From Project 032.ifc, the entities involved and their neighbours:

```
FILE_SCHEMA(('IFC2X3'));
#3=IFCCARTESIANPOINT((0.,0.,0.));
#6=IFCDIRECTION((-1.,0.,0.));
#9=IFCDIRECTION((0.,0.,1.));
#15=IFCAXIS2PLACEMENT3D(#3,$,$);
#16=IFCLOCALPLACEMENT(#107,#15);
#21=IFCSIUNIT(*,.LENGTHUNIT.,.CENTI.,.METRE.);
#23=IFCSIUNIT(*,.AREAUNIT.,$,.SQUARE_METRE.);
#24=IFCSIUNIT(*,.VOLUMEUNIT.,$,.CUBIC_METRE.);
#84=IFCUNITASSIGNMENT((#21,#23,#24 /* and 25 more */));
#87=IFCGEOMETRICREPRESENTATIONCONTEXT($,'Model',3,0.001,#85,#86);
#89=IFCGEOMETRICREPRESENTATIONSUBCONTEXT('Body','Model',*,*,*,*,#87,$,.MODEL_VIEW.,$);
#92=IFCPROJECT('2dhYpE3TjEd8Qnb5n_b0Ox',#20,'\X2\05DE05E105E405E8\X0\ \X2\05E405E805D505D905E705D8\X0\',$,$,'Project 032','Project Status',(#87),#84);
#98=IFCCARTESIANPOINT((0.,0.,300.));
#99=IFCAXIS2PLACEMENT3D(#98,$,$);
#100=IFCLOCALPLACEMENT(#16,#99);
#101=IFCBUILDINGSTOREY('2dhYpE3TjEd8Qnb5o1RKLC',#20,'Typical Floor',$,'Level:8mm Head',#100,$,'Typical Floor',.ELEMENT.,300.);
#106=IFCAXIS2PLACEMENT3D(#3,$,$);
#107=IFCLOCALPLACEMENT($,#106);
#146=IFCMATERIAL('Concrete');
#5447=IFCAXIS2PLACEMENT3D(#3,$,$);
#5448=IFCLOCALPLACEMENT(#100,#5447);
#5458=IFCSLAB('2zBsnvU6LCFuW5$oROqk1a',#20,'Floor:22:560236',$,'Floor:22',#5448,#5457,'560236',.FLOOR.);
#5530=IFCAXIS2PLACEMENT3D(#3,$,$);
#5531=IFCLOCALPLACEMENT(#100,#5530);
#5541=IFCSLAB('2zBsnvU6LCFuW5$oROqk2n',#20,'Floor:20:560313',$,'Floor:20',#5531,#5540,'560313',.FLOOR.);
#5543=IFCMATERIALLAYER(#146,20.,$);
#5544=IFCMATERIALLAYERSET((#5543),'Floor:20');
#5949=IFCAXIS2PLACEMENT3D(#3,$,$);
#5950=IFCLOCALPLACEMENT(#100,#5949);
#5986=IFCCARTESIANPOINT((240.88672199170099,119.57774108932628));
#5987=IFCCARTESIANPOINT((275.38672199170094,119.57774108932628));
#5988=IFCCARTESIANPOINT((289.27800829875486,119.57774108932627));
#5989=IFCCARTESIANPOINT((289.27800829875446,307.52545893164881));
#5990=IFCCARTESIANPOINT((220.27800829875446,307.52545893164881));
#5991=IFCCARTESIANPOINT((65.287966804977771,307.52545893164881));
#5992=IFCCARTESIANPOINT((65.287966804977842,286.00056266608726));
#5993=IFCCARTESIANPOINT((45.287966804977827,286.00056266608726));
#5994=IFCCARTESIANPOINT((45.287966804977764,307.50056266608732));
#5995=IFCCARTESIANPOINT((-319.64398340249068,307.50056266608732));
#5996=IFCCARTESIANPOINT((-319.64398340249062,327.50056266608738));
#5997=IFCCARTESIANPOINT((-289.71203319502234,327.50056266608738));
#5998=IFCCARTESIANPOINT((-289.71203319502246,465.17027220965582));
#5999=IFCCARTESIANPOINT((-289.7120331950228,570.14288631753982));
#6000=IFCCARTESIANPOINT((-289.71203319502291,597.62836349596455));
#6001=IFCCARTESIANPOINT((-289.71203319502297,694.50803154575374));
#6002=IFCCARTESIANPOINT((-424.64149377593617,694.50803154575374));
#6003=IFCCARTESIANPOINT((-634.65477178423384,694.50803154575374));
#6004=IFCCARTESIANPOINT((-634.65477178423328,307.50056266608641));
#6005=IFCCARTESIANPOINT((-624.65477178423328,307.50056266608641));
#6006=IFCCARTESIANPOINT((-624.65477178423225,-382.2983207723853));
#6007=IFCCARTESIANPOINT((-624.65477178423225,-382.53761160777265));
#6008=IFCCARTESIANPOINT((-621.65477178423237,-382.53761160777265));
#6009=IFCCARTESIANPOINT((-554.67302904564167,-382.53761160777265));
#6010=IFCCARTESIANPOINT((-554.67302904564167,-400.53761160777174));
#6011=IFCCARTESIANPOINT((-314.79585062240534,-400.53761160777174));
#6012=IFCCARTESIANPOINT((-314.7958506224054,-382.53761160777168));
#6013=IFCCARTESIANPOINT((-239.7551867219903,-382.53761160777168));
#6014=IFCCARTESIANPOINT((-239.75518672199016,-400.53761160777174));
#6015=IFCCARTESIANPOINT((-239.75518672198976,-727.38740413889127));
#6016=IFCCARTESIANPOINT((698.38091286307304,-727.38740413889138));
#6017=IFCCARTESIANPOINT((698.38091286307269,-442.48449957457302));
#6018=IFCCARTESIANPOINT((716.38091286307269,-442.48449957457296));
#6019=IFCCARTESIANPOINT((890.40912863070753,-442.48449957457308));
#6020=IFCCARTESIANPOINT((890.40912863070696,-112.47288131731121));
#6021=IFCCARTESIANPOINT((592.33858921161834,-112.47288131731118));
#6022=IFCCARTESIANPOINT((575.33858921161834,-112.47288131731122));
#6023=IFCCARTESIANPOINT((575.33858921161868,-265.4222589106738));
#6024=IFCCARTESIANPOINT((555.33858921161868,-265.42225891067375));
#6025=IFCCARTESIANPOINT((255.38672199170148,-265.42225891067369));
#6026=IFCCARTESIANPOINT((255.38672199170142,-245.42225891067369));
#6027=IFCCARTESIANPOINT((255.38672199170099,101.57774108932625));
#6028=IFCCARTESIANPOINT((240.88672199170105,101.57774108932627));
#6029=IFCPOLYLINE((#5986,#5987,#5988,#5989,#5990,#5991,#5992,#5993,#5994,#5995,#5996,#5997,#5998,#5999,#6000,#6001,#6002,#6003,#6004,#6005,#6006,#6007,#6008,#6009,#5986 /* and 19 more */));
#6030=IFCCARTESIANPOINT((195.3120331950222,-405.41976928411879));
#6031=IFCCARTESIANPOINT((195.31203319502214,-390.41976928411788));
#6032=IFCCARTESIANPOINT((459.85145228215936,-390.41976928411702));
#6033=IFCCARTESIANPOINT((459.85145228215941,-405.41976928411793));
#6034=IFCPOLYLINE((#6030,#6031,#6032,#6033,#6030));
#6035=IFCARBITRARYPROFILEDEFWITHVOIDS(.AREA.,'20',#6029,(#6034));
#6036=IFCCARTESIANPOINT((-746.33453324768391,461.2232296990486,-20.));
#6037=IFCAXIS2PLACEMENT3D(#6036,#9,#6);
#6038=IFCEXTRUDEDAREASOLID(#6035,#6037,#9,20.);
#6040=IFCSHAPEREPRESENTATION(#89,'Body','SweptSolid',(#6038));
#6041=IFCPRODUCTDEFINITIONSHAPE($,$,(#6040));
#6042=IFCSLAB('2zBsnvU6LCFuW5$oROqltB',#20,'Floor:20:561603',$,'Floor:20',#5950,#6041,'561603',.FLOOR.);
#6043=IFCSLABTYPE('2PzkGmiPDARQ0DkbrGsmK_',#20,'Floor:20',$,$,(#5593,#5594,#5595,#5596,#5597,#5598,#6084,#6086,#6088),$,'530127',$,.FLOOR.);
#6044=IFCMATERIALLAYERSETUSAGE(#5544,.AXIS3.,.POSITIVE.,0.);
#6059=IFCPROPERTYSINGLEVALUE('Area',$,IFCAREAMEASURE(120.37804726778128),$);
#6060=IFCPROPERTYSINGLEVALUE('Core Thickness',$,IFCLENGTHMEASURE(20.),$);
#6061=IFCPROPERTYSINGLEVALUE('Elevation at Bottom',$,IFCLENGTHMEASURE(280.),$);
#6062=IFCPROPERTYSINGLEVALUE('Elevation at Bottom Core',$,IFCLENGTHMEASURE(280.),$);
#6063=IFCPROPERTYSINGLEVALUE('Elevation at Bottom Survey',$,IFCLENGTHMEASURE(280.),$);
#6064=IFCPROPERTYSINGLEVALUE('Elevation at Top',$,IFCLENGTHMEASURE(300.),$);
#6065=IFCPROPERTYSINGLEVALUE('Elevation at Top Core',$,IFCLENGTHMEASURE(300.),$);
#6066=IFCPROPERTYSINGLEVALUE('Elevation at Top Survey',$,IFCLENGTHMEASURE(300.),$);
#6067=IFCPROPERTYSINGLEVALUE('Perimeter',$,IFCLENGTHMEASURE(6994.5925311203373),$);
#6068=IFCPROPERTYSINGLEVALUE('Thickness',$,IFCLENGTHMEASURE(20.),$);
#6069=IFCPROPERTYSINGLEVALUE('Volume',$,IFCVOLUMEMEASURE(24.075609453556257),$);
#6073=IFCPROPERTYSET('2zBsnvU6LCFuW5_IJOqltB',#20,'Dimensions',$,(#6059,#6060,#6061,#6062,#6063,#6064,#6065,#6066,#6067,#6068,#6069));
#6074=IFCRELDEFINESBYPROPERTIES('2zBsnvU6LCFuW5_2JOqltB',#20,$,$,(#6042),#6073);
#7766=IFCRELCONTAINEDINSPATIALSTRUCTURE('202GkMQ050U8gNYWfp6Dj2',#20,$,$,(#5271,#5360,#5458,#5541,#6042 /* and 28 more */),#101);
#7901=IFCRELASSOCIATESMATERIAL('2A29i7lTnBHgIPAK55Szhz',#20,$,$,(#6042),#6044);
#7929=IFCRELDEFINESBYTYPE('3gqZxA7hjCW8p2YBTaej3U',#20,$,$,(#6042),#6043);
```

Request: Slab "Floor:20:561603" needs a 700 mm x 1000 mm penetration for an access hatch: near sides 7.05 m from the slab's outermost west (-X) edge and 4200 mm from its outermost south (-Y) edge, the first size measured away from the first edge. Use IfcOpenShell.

```python
import numpy as np
import ifcopenshell
import ifcopenshell.api.feature
import ifcopenshell.api.geometry
import ifcopenshell.api.pset
import ifcopenshell.api.root
import ifcopenshell.geom
import ifcopenshell.util.element
import ifcopenshell.util.placement
import ifcopenshell.util.representation
import ifcopenshell.util.shape
import ifcopenshell.util.unit

model = ifcopenshell.open("Project 032.ifc")
unit_scale = ifcopenshell.util.unit.calculate_unit_scale(model)
area_scale = ifcopenshell.util.unit.calculate_unit_scale(model, "AREAUNIT")
volume_scale = ifcopenshell.util.unit.calculate_unit_scale(model, "VOLUMEUNIT")
settings = ifcopenshell.geom.settings()


def volume(element):
    """Net volume in cubic metres, openings subtracted."""
    shape = ifcopenshell.geom.create_shape(settings, element)
    return ifcopenshell.util.shape.get_volume(shape.geometry)


slab = model.by_id(6042)
before = volume(slab)

# Extent in the slab's own axes, in metres. The edges named are its -X and -Y sides.
slab_shape = ifcopenshell.geom.create_shape(settings, slab)
vertices = ifcopenshell.util.shape.get_vertices(slab_shape.geometry)
x_min, y_min, bottom = vertices.min(axis=0)
top = vertices[:, 2].max()

opening = ifcopenshell.api.root.create_entity(model, ifc_class="IfcOpeningElement", name="Access hatch opening")
context = ifcopenshell.util.representation.get_context(model, "Model", "Body", "MODEL_VIEW")
width, depth = 0.7, 1
outline = [(0.0, 0.0), (width, 0.0), (width, depth), (0.0, depth), (0.0, 0.0)]
# Overshoot both faces by 50 mm so the cut is clean.
shape = ifcopenshell.api.geometry.add_slab_representation(
    model, context=context, depth=top - bottom + 0.1, polyline=outline
)
ifcopenshell.api.geometry.assign_representation(model, product=opening, representation=shape)

matrix = ifcopenshell.util.placement.get_local_placement(slab.ObjectPlacement)
matrix[:, 3] = matrix @ np.append(np.array([x_min + 7.05, y_min + 4.2, bottom - 0.05]) / unit_scale, 1.0)
ifcopenshell.api.geometry.edit_object_placement(model, product=opening, matrix=matrix, is_si=False)
ifcopenshell.api.feature.add_feature(model, feature=opening, element=slab)

after = volume(slab)

# Update the slab's stored quantities.
pset = model.by_id(ifcopenshell.util.element.get_pset(slab, "Dimensions", should_inherit=False)["id"])
ifcopenshell.api.pset.edit_pset(model, pset=pset, properties={
    "Area": model.create_entity("IfcAreaMeasure", after / (top - bottom) / area_scale),
    "Volume": model.create_entity("IfcVolumeMeasure", after / volume_scale),
})

print(f"slab volume {before:.3f} -> {after:.3f} m3")

model.write("Project 032_edited.ifc")
```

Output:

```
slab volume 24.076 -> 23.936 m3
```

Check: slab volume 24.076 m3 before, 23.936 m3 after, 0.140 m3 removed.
